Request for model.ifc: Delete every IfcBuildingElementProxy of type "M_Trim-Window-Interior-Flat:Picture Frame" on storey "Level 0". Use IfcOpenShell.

First a look at what the model holds.

```python
import ifcopenshell
import ifcopenshell.util.element

model = ifcopenshell.open("model.ifc")
print(model.schema)
storey = next(s for s in model.by_type("IfcBuildingStorey") if s.Name == "Level 0")
proxies = [e for e in ifcopenshell.util.element.get_decomposition(storey) if e.is_a("IfcBuildingElementProxy")]
seen = {}
for e in proxies:
    element_type = ifcopenshell.util.element.get_type(e)
    name = element_type.Name if element_type not in (None, e) else None
    seen[name] = seen.get(name, 0) + 1
for name, count in sorted(seen.items(), key=str):
    print(count, "x", name)
```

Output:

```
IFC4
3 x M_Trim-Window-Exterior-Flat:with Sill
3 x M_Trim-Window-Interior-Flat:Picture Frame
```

```python
import ifcopenshell
import ifcopenshell.api.root
import ifcopenshell.util.element

model = ifcopenshell.open("model.ifc")

storey = next(s for s in model.by_type("IfcBuildingStorey") if s.Name == "Level 0")
proxies = [e for e in ifcopenshell.util.element.get_decomposition(storey) if e.is_a("IfcBuildingElementProxy")]
targets = [e for e in proxies if (t := ifcopenshell.util.element.get_type(e)) not in (None, e) and t.Name == "M_Trim-Window-Interior-Flat:Picture Frame"]

for e in targets:
    ifcopenshell.api.root.remove_product(model, product=e)
print(len(targets), "removed")

model.write("model_v2.ifc")
```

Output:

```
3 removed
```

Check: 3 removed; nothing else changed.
